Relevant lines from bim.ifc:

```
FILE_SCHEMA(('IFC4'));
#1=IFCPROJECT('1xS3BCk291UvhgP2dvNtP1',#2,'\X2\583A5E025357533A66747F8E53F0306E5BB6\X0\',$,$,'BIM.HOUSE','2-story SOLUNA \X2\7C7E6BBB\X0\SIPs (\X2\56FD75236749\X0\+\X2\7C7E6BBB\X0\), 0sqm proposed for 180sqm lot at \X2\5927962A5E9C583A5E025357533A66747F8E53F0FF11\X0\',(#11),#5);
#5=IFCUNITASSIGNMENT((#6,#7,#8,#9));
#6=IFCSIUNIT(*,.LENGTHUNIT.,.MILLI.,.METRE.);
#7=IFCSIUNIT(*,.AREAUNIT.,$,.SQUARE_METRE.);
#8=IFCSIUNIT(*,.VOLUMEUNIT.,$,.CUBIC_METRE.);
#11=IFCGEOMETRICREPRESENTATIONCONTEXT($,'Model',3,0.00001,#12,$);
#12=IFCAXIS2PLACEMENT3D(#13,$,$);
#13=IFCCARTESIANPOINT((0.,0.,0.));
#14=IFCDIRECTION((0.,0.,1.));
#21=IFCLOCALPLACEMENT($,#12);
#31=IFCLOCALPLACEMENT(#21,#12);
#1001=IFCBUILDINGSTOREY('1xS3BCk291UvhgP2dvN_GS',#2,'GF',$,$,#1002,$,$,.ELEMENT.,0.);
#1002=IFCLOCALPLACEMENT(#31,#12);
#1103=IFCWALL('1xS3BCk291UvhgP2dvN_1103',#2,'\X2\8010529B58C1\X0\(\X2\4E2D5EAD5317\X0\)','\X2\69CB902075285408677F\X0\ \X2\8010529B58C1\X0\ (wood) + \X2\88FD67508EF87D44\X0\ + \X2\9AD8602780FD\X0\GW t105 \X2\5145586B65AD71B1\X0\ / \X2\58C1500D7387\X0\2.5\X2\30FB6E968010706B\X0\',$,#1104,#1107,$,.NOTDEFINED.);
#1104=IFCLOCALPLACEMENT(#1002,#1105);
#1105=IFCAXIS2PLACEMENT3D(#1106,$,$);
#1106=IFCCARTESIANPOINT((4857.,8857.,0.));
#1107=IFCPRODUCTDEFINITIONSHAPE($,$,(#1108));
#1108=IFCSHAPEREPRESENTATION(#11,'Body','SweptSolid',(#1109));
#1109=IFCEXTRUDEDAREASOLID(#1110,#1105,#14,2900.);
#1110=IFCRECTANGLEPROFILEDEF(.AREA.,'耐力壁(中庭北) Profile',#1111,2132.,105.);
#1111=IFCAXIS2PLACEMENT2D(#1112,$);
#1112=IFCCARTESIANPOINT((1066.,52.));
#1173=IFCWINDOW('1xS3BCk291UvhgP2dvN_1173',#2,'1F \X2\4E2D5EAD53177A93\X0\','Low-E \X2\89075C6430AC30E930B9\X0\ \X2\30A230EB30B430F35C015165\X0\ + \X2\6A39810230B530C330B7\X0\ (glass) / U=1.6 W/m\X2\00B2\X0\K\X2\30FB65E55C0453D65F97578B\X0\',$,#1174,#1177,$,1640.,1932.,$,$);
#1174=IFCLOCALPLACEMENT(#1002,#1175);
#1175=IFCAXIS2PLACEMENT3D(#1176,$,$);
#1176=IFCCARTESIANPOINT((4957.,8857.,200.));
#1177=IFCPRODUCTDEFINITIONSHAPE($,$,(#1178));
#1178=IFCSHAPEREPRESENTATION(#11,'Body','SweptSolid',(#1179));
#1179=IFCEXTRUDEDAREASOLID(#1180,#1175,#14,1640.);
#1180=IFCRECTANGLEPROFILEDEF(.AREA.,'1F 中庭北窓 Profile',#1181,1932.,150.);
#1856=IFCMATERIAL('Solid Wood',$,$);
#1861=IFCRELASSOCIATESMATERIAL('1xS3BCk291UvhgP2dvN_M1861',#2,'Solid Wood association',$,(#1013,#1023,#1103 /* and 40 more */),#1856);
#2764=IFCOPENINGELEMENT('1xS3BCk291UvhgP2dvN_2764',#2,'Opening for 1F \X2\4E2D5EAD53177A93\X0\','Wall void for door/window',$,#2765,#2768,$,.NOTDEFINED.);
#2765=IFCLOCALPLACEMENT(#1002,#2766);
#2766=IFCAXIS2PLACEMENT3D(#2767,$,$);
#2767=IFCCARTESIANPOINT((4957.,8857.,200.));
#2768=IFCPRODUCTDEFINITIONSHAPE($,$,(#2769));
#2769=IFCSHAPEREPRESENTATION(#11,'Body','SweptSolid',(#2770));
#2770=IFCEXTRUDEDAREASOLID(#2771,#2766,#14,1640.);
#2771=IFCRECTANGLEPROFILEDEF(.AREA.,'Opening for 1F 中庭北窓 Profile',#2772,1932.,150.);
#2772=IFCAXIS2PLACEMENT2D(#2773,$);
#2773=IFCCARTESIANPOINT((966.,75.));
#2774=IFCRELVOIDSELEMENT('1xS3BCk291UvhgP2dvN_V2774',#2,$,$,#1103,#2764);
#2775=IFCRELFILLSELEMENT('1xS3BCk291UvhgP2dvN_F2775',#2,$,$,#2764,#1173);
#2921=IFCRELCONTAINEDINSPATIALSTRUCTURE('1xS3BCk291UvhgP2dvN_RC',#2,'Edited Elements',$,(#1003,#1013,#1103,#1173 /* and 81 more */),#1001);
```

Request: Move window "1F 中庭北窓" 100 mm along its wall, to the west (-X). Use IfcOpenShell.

```python
import ifcopenshell
import ifcopenshell.api.geometry
import ifcopenshell.util.placement
import ifcopenshell.util.unit

model = ifcopenshell.open("bim.ifc")
unit_scale = ifcopenshell.util.unit.calculate_unit_scale(model)

window = model.by_guid("1xS3BCk291UvhgP2dvN_1173")
opening = window.FillsVoids[0].RelatingOpeningElement
wall = opening.VoidsElements[0].RelatingBuildingElement

wall_matrix = ifcopenshell.util.placement.get_local_placement(wall.ObjectPlacement)
shift = wall_matrix[:3, 0] * -0.1 / unit_scale
before = ifcopenshell.util.placement.get_local_placement(window.ObjectPlacement)[:3, 3].copy()

# The window is not placed relative to its opening, so move both.
for product in (opening, window):
    matrix = ifcopenshell.util.placement.get_local_placement(product.ObjectPlacement)
    matrix[:3, 3] += shift
    ifcopenshell.api.geometry.edit_object_placement(model, product=product, matrix=matrix, is_si=False)

after = ifcopenshell.util.placement.get_local_placement(window.ObjectPlacement)[:3, 3]
print("window moved by", (after - before).round(3) + 0.0)

model.write("bim_rev.ifc")
```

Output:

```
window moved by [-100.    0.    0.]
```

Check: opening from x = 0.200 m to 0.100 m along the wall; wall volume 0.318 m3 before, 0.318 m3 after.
